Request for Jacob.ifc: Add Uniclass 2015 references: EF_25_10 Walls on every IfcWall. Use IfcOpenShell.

First a look at what the model holds.

```python
import ifcopenshell

model = ifcopenshell.open("Jacob.ifc")
print(model.schema)
print("classifications:", [c.Name for c in model.by_type("IfcClassification")])
for ifc_class in ("IfcDoor", "IfcRoof", "IfcStair", "IfcWall", "IfcWindow"):
    print(ifc_class, len(model.by_type(ifc_class)))
```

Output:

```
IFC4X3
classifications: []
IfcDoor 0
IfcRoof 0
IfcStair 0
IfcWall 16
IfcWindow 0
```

```python
import ifcopenshell
import ifcopenshell.api.classification

model = ifcopenshell.open("Jacob.ifc")

system = ifcopenshell.api.classification.add_classification(model, classification="Uniclass 2015")

codes = {
    "IfcWall": ("EF_25_10", "Walls"),
}
for ifc_class, (code, name) in codes.items():
    products = model.by_type(ifc_class)
    ifcopenshell.api.classification.add_reference(
        model, products=products, classification=system, identification=code, name=name
    )
    print(code, len(products))

model.write("Jacob_updated.ifc")
```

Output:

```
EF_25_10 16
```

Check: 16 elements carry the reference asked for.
